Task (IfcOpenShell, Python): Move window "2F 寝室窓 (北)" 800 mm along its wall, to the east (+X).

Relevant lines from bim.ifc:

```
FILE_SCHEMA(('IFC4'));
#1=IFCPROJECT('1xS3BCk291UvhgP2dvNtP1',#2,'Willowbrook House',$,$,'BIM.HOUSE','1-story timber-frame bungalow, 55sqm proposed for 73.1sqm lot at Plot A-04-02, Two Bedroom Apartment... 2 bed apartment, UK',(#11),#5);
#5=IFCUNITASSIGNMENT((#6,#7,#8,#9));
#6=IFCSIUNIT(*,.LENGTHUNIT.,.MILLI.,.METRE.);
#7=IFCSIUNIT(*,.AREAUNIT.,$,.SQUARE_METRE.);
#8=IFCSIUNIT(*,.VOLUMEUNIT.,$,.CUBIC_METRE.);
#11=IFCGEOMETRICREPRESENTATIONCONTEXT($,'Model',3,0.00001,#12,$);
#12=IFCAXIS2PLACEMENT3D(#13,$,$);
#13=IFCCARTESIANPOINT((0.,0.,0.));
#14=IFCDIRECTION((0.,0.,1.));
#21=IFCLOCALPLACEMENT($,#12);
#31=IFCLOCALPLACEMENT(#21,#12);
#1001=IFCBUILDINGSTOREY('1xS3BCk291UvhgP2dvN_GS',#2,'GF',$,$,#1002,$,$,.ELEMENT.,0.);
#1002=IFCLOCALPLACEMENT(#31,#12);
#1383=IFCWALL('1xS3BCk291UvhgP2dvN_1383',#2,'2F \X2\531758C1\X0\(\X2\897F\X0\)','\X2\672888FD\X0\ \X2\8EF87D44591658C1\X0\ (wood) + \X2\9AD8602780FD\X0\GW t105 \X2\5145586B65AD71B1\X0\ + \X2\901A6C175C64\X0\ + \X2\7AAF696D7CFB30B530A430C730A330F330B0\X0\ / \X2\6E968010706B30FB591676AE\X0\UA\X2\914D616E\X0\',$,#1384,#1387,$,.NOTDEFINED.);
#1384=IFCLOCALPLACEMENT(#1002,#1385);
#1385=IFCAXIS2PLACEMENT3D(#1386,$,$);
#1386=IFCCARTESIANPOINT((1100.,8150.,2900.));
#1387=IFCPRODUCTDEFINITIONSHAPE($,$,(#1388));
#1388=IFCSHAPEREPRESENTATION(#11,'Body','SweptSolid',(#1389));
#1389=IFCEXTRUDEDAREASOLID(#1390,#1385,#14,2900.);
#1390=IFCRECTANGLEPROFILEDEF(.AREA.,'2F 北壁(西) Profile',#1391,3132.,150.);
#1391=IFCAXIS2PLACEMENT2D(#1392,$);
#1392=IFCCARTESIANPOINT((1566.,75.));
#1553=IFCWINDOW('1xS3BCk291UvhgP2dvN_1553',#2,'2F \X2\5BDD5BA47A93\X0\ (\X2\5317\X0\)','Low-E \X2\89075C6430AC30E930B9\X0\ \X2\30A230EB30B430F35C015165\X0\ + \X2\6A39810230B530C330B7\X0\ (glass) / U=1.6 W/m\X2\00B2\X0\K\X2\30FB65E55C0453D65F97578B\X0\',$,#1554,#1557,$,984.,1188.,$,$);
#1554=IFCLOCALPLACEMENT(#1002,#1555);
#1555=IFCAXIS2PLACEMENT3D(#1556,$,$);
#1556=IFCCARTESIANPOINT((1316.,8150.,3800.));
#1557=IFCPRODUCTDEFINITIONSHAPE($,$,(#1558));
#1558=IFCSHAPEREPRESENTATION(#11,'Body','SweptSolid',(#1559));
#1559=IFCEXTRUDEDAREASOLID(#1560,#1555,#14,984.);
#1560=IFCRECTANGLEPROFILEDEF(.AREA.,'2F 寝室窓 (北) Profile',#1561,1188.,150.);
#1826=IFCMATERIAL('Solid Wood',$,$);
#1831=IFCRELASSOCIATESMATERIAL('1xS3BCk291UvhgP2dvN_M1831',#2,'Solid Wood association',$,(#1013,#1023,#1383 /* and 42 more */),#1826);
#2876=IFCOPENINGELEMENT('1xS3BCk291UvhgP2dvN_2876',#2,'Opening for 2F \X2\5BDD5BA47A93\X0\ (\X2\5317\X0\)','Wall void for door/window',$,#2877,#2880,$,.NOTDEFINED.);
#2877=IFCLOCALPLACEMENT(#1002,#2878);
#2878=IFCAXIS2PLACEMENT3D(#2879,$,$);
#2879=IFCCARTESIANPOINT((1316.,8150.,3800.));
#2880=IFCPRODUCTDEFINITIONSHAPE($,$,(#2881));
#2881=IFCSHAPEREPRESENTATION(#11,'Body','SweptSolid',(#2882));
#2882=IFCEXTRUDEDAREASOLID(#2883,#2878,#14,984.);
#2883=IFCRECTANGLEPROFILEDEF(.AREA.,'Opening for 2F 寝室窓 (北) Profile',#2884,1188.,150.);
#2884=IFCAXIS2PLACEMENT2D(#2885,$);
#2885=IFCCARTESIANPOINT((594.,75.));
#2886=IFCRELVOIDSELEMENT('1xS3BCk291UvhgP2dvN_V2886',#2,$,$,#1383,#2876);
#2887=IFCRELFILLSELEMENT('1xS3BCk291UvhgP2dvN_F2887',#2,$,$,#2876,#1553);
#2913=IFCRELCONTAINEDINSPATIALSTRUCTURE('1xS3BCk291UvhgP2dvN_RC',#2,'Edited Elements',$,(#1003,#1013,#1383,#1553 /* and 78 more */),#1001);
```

```python
import ifcopenshell
import ifcopenshell.api.geometry
import ifcopenshell.util.placement

model = ifcopenshell.open("bim.ifc")

window = model.by_guid("1xS3BCk291UvhgP2dvN_1553")
opening = window.FillsVoids[0].RelatingOpeningElement
wall = opening.VoidsElements[0].RelatingBuildingElement

wall_matrix = ifcopenshell.util.placement.get_local_placement(wall.ObjectPlacement)
shift = wall_matrix[:3, 0] * 800.0
before = ifcopenshell.util.placement.get_local_placement(window.ObjectPlacement)[:3, 3].copy()

# The window is not placed relative to its opening, so move both.
for product in (opening, window):
    matrix = ifcopenshell.util.placement.get_local_placement(product.ObjectPlacement)
    matrix[:3, 3] += shift
    ifcopenshell.api.geometry.edit_object_placement(model, product=product, matrix=matrix, is_si=False)

after = ifcopenshell.util.placement.get_local_placement(window.ObjectPlacement)[:3, 3]
print("window moved by", (after - before).round(3) + 0.0)

model.write("bim_updated.ifc")
```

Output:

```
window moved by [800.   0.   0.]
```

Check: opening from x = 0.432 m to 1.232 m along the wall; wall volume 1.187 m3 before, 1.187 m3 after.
